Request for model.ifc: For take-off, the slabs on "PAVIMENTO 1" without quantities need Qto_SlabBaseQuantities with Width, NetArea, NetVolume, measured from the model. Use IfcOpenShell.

First a look at what the model holds.

```python
import ifcopenshell
import ifcopenshell.util.element
import ifcopenshell.util.unit

model = ifcopenshell.open("model.ifc")
print(model.schema)
for unit_type in ("LENGTHUNIT", "AREAUNIT", "VOLUMEUNIT"):
    print(unit_type, ifcopenshell.util.unit.calculate_unit_scale(model, unit_type))
storey = next(s for s in model.by_type("IfcBuildingStorey") if s.Name == "PAVIMENTO 1")
slabs = [e for e in ifcopenshell.util.element.get_decomposition(storey) if e.is_a("IfcSlab")]
for e in sorted(slabs, key=lambda e: e.id()):
    print(e.id(), e.is_a(), e.Name, list(ifcopenshell.util.element.get_psets(e, qtos_only=True)), sep=" | ")
```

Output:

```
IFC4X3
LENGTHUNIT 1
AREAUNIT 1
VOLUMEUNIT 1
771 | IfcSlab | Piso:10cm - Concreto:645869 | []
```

```python
import ifcopenshell
import ifcopenshell.api.pset
import ifcopenshell.geom
import ifcopenshell.util.element
import ifcopenshell.util.shape
import ifcopenshell.util.unit

model = ifcopenshell.open("model.ifc")
unit_scale = ifcopenshell.util.unit.calculate_unit_scale(model)
area_scale = ifcopenshell.util.unit.calculate_unit_scale(model, "AREAUNIT")
volume_scale = ifcopenshell.util.unit.calculate_unit_scale(model, "VOLUMEUNIT")
settings = ifcopenshell.geom.settings()

storey = next(s for s in model.by_type("IfcBuildingStorey") if s.Name == "PAVIMENTO 1")
slabs = [e for e in ifcopenshell.util.element.get_decomposition(storey) if e.is_a("IfcSlab")]

for e in sorted(slabs, key=lambda e: e.id()):
    if ifcopenshell.util.element.get_psets(e, qtos_only=True, should_inherit=False):
        continue
    # Geometry comes back in metres, in the element's own axes.
    shape = ifcopenshell.geom.create_shape(settings, e)
    values = {
        "Width": ifcopenshell.util.shape.get_z(shape.geometry) / unit_scale,
        "NetArea": ifcopenshell.util.shape.get_footprint_area(shape.geometry) / area_scale,
        "NetVolume": ifcopenshell.util.shape.get_volume(shape.geometry) / volume_scale,
    }
    qto = ifcopenshell.api.pset.add_qto(model, product=e, name="Qto_SlabBaseQuantities")
    ifcopenshell.api.pset.edit_qto(model, qto=qto, properties=values)
    print(e.id(), {k: round(v, 3) for k, v in values.items()})

model.write("model_updated.ifc")
```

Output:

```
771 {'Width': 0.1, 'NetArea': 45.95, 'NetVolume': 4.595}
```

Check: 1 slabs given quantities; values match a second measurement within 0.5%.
